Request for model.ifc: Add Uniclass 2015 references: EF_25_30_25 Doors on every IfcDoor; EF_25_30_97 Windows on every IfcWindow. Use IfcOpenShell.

First a look at what the model holds.

```python
import ifcopenshell

model = ifcopenshell.open("model.ifc")
print(model.schema)
print("classifications:", [c.Name for c in model.by_type("IfcClassification")])
for ifc_class in ("IfcDoor", "IfcRoof", "IfcStair", "IfcWall", "IfcWindow"):
    print(ifc_class, len(model.by_type(ifc_class)))
```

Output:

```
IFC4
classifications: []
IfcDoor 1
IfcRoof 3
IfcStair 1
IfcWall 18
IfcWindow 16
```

```python
import ifcopenshell
import ifcopenshell.api.classification

model = ifcopenshell.open("model.ifc")

system = ifcopenshell.api.classification.add_classification(model, classification="Uniclass 2015")

codes = {
    "IfcDoor": ("EF_25_30_25", "Doors"),
    "IfcWindow": ("EF_25_30_97", "Windows"),
}
for ifc_class, (code, name) in codes.items():
    products = model.by_type(ifc_class)
    ifcopenshell.api.classification.add_reference(
        model, products=products, classification=system, identification=code, name=name
    )
    print(code, len(products))

model.write("model_edited.ifc")
```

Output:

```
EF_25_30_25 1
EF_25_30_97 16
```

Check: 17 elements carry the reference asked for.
